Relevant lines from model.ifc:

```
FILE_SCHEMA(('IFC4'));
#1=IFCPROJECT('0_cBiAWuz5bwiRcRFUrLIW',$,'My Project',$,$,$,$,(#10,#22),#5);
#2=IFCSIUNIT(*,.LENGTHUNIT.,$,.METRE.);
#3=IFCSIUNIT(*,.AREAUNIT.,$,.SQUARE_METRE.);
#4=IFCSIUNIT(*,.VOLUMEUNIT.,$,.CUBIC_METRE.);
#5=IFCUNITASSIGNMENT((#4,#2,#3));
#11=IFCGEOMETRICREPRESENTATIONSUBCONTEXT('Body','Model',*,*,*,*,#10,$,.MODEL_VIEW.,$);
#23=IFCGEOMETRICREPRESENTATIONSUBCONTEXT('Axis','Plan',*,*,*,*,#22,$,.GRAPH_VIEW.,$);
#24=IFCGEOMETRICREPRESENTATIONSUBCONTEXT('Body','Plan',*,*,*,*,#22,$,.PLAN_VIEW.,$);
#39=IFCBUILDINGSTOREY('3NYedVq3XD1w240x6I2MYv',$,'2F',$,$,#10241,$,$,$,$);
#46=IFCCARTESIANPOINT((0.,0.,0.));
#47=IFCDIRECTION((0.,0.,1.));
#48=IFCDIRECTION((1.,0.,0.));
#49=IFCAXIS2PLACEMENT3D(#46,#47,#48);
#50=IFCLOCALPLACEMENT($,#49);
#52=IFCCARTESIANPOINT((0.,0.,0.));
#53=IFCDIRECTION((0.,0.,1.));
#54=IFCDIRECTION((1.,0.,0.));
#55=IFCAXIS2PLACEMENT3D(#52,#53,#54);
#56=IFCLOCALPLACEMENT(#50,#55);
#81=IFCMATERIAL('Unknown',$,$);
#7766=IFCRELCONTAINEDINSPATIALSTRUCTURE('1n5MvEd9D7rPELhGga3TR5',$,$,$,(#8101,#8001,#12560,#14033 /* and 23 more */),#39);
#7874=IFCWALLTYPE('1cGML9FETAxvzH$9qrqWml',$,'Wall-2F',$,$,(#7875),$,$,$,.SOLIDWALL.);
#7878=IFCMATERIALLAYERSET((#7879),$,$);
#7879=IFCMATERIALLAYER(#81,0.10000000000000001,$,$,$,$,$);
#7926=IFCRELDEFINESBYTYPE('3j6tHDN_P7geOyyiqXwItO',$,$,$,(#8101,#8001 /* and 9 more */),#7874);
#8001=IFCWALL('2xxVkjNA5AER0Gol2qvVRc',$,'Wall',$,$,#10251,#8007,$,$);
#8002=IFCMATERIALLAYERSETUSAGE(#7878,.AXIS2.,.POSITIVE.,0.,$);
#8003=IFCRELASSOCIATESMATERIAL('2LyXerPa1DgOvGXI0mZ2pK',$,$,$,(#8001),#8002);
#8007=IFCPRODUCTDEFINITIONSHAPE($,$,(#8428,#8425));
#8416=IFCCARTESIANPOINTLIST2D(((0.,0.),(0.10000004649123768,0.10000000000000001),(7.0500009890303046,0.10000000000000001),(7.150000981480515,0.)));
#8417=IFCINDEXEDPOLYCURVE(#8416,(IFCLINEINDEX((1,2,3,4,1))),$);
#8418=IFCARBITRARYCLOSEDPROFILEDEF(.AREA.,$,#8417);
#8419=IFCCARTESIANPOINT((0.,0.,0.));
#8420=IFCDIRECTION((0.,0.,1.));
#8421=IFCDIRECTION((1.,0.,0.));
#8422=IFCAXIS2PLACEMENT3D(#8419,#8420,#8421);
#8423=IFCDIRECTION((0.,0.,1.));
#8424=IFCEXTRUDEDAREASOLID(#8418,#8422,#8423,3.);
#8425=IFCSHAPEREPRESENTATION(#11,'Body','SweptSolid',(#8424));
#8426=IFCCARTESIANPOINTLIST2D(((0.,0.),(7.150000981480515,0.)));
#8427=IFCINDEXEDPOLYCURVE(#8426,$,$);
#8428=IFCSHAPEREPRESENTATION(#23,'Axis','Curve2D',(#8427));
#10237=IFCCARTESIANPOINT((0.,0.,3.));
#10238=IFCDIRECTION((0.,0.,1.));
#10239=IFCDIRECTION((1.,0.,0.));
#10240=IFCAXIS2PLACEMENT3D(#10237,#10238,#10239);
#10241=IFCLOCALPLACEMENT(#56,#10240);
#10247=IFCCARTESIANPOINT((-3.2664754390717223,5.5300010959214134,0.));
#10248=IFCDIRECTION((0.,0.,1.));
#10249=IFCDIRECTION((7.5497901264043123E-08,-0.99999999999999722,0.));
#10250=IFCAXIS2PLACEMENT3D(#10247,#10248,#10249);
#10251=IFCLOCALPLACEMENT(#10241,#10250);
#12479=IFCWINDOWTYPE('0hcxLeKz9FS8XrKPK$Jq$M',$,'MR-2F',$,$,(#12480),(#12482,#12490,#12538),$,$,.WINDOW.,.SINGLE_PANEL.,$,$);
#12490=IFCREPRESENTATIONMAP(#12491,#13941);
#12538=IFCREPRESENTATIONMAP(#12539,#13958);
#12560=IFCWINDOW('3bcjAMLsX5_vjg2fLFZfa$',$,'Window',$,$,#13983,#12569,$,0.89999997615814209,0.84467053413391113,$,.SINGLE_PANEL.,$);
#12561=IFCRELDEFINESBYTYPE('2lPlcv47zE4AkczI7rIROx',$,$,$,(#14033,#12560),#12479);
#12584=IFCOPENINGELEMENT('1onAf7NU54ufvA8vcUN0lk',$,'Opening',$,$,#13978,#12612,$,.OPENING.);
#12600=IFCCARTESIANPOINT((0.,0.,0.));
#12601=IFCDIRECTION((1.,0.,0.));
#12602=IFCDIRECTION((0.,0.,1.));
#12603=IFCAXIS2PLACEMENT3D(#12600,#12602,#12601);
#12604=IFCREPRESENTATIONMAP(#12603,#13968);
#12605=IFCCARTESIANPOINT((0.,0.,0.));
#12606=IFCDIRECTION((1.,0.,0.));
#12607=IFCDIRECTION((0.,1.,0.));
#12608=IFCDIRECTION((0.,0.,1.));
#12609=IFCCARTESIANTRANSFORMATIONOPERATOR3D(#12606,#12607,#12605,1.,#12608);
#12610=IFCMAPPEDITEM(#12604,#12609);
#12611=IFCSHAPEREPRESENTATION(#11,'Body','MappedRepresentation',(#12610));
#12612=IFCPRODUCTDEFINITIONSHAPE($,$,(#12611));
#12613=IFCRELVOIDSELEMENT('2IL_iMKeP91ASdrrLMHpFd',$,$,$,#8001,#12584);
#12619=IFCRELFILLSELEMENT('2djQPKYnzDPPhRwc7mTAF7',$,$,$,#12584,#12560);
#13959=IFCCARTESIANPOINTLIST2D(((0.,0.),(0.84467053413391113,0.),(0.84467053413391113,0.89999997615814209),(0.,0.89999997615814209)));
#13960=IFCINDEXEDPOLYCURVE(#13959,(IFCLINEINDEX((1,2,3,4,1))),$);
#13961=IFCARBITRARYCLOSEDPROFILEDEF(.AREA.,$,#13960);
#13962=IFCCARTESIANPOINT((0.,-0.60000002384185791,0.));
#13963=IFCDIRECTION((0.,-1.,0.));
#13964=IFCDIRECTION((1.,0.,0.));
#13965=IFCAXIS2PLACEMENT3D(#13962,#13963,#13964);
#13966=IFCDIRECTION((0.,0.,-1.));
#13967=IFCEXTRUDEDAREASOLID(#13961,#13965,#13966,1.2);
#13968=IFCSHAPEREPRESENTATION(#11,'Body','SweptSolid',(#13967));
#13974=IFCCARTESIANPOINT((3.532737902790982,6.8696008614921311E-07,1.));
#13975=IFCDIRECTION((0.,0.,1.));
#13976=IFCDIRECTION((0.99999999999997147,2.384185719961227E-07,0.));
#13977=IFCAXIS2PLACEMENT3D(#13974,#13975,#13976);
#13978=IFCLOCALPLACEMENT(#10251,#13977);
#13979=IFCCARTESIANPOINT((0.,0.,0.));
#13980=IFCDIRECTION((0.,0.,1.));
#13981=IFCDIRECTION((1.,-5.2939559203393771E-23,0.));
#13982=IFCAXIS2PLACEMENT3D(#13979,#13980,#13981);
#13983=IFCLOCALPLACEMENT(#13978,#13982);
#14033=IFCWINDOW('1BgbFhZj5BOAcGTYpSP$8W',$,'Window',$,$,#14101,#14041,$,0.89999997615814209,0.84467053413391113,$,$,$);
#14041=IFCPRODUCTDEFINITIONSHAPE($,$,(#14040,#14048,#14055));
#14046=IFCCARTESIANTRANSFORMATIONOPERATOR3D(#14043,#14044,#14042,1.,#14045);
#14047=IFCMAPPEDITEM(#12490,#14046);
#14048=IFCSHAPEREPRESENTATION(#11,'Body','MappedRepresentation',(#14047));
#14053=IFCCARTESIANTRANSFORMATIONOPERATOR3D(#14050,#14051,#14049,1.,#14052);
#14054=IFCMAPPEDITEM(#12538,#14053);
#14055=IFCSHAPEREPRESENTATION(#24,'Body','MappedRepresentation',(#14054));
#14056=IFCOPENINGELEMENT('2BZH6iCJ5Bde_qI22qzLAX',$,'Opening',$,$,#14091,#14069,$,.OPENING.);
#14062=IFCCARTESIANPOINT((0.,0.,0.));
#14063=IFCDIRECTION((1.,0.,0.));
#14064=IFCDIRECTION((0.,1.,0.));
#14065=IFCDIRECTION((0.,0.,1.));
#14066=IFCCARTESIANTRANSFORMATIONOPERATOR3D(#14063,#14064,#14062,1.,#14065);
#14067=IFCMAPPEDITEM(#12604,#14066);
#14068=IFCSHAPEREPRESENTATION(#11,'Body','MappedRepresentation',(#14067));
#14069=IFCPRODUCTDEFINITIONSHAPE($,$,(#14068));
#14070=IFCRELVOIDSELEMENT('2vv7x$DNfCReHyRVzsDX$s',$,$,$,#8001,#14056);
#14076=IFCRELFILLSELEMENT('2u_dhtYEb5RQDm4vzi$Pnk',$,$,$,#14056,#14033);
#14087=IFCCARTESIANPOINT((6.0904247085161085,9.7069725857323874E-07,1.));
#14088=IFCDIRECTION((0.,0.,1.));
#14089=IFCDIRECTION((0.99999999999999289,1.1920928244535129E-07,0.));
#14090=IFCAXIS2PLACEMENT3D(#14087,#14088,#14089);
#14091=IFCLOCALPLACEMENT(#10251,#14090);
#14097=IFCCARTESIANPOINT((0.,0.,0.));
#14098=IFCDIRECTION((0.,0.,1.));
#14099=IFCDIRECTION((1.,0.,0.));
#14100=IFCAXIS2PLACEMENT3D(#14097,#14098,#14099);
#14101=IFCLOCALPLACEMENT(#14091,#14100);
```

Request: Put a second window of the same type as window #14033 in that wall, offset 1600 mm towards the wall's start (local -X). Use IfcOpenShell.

```python
import ifcopenshell
import ifcopenshell.api.feature
import ifcopenshell.api.geometry
import ifcopenshell.api.root
import ifcopenshell.geom
import ifcopenshell.util.element
import ifcopenshell.util.placement
import ifcopenshell.util.shape

model = ifcopenshell.open("model.ifc")
settings = ifcopenshell.geom.settings()


def volume(element):
    """Net volume in cubic metres, openings subtracted."""
    shape = ifcopenshell.geom.create_shape(settings, element)
    return ifcopenshell.util.shape.get_volume(shape.geometry)


window = model.by_guid("1BgbFhZj5BOAcGTYpSP$8W")
opening = window.FillsVoids[0].RelatingOpeningElement
wall = opening.VoidsElements[0].RelatingBuildingElement
before = volume(wall)
shift = ifcopenshell.util.placement.get_local_placement(wall.ObjectPlacement)[:3, 0] * -1.6

# copy_class copies the void relationship, type, container and properties, but no geometry.
new_opening = ifcopenshell.api.root.copy_class(model, product=opening)
new_opening.Representation = ifcopenshell.util.element.copy_deep(
    model, opening.Representation, exclude=["IfcGeometricRepresentationContext", "IfcRepresentationMap"]
)
new_window = ifcopenshell.api.root.copy_class(model, product=window)
new_window.Representation = ifcopenshell.util.element.copy_deep(
    model, window.Representation, exclude=["IfcGeometricRepresentationContext", "IfcRepresentationMap"]
)
ifcopenshell.api.feature.add_filling(model, opening=new_opening, element=new_window)

for old, new in ((opening, new_opening), (window, new_window)):
    matrix = ifcopenshell.util.placement.get_local_placement(old.ObjectPlacement)
    matrix[:3, 3] += shift
    ifcopenshell.api.geometry.edit_object_placement(model, product=new, matrix=matrix, is_si=False)

after = volume(wall)

print(f"wall volume {before:.3f} -> {after:.3f} m3")

model.write("model-out.ifc")
```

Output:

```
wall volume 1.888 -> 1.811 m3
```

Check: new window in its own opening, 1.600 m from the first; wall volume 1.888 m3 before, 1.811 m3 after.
